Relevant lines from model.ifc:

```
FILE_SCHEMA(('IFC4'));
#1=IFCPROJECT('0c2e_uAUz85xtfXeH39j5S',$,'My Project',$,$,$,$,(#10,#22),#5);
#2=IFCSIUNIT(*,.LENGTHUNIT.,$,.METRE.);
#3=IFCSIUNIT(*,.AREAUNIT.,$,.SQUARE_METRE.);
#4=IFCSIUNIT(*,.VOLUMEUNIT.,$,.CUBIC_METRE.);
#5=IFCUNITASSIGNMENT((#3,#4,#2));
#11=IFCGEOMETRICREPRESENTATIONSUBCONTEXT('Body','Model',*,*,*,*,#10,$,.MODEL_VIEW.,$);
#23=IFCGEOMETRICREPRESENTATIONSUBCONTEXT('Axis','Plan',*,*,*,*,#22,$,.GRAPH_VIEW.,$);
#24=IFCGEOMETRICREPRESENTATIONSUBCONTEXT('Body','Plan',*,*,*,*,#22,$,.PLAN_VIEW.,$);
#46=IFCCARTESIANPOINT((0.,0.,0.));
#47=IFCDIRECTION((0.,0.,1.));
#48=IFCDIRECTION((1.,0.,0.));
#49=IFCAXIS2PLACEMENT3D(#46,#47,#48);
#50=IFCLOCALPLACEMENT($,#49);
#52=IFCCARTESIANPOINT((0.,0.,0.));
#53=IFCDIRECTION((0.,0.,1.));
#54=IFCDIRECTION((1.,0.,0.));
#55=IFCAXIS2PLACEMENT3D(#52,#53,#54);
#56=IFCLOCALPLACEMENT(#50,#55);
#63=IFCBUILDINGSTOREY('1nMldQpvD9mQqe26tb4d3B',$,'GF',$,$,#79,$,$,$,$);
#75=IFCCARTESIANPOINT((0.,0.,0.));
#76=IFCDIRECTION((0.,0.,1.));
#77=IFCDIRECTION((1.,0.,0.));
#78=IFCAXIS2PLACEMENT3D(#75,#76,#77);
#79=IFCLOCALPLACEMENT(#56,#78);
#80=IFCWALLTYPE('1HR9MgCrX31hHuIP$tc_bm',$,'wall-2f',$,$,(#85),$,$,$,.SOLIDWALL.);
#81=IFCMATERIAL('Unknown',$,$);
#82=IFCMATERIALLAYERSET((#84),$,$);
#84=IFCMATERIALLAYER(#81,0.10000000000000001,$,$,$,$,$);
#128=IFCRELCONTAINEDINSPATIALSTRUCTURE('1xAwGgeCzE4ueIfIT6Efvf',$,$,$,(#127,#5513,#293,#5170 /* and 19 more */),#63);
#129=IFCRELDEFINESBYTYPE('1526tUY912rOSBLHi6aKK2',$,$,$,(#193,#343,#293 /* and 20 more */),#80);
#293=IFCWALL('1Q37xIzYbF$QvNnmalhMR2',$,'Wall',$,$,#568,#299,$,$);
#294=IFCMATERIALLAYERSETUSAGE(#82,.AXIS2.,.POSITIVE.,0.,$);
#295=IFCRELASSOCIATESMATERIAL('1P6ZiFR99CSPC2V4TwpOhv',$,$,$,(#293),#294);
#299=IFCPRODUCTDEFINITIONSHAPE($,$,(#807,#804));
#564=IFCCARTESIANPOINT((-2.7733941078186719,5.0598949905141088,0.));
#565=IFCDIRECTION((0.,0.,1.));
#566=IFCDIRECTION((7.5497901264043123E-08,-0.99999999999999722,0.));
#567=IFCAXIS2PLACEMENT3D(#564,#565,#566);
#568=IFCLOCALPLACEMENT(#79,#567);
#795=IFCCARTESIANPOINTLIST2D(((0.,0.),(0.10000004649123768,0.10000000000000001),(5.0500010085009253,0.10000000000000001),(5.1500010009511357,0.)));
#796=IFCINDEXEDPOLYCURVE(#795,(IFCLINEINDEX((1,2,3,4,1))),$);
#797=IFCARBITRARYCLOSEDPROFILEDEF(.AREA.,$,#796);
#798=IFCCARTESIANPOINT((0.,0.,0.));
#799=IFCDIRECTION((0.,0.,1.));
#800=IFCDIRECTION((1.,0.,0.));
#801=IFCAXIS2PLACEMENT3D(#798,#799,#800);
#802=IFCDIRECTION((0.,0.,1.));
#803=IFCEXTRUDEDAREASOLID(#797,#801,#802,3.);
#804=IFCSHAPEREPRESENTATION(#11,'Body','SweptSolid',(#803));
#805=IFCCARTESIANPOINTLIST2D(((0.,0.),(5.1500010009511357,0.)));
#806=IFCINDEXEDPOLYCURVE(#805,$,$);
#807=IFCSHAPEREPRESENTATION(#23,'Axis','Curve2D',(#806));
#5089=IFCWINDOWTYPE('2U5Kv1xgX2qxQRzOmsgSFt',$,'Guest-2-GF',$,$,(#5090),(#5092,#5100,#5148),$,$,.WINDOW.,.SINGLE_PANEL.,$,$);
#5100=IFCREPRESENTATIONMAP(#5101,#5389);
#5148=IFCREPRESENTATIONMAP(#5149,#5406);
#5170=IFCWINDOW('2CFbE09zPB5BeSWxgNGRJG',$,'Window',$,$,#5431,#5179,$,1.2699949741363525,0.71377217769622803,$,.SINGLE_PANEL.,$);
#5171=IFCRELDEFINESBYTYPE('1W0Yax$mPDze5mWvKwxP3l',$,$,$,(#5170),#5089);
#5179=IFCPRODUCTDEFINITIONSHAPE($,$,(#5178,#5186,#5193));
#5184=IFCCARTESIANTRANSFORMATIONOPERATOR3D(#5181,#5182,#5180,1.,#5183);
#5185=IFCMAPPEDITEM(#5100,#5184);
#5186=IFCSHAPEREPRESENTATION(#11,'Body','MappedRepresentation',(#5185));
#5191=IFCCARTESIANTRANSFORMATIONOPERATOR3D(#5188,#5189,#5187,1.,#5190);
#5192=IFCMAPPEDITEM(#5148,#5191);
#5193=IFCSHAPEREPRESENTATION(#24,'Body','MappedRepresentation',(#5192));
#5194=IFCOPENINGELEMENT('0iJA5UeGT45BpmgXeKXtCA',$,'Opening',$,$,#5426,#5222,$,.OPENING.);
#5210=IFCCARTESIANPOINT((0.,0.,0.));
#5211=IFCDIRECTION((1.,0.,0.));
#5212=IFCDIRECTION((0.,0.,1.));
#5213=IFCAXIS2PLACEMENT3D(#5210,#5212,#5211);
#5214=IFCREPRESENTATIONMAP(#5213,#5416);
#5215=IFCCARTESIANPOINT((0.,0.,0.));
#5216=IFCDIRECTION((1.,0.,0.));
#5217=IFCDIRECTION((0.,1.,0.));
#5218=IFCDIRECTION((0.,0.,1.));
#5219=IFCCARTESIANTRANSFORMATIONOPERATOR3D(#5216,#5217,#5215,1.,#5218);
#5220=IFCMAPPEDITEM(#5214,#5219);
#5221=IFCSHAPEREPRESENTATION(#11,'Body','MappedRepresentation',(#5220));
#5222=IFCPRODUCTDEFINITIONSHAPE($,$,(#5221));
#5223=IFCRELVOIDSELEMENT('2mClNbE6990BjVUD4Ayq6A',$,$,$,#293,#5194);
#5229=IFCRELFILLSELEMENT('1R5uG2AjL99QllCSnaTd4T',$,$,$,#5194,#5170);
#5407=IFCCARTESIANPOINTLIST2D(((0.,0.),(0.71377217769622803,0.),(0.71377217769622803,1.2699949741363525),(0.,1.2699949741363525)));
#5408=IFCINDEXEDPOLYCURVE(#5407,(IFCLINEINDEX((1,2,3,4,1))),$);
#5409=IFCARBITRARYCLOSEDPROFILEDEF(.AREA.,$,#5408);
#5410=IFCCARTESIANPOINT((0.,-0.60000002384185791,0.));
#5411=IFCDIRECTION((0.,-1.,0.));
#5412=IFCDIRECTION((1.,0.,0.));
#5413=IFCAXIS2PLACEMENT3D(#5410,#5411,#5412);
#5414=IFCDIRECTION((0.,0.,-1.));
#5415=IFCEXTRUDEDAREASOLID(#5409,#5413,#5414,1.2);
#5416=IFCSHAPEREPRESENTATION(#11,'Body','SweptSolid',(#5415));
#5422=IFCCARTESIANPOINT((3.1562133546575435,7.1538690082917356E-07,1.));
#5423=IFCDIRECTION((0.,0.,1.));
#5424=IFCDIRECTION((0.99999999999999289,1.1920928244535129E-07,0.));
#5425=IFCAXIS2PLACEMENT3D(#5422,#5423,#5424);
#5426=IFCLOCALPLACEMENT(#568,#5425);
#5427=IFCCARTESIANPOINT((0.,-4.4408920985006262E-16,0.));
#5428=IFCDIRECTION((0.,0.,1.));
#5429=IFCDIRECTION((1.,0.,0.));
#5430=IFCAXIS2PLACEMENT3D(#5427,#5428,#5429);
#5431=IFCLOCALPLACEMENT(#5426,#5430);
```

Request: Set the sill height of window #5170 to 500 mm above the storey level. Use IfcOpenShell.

```python
import numpy as np
import ifcopenshell
import ifcopenshell.api.geometry
import ifcopenshell.geom
import ifcopenshell.util.element
import ifcopenshell.util.placement
import ifcopenshell.util.shape
import ifcopenshell.util.unit

model = ifcopenshell.open("model.ifc")
unit_scale = ifcopenshell.util.unit.calculate_unit_scale(model)

window = model.by_id(5170)
opening = window.FillsVoids[0].RelatingOpeningElement
storey = ifcopenshell.util.element.get_container(window, ifc_class="IfcBuildingStorey")
level = ifcopenshell.util.placement.get_local_placement(storey.ObjectPlacement)[2, 3]

# The opening's origin need not be at the sill, so measure its lowest point.
shape = ifcopenshell.geom.create_shape(ifcopenshell.geom.settings(), opening)
bottom = ifcopenshell.util.shape.get_shape_bottom_elevation(shape, shape.geometry) / unit_scale
dz = level + 0.5 - bottom

shift = np.array([0.0, 0.0, dz])
# The window is placed relative to its opening, so it follows when the opening moves.
matrix = ifcopenshell.util.placement.get_local_placement(opening.ObjectPlacement)
matrix[:3, 3] += shift
ifcopenshell.api.geometry.edit_object_placement(
    model, product=opening, matrix=matrix, is_si=False, should_transform_children=True
)

print(f"moved by {dz * unit_scale:+.3f} m")

model.write("model_rev.ifc")
```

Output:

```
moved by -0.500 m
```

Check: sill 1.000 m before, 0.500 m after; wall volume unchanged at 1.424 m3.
